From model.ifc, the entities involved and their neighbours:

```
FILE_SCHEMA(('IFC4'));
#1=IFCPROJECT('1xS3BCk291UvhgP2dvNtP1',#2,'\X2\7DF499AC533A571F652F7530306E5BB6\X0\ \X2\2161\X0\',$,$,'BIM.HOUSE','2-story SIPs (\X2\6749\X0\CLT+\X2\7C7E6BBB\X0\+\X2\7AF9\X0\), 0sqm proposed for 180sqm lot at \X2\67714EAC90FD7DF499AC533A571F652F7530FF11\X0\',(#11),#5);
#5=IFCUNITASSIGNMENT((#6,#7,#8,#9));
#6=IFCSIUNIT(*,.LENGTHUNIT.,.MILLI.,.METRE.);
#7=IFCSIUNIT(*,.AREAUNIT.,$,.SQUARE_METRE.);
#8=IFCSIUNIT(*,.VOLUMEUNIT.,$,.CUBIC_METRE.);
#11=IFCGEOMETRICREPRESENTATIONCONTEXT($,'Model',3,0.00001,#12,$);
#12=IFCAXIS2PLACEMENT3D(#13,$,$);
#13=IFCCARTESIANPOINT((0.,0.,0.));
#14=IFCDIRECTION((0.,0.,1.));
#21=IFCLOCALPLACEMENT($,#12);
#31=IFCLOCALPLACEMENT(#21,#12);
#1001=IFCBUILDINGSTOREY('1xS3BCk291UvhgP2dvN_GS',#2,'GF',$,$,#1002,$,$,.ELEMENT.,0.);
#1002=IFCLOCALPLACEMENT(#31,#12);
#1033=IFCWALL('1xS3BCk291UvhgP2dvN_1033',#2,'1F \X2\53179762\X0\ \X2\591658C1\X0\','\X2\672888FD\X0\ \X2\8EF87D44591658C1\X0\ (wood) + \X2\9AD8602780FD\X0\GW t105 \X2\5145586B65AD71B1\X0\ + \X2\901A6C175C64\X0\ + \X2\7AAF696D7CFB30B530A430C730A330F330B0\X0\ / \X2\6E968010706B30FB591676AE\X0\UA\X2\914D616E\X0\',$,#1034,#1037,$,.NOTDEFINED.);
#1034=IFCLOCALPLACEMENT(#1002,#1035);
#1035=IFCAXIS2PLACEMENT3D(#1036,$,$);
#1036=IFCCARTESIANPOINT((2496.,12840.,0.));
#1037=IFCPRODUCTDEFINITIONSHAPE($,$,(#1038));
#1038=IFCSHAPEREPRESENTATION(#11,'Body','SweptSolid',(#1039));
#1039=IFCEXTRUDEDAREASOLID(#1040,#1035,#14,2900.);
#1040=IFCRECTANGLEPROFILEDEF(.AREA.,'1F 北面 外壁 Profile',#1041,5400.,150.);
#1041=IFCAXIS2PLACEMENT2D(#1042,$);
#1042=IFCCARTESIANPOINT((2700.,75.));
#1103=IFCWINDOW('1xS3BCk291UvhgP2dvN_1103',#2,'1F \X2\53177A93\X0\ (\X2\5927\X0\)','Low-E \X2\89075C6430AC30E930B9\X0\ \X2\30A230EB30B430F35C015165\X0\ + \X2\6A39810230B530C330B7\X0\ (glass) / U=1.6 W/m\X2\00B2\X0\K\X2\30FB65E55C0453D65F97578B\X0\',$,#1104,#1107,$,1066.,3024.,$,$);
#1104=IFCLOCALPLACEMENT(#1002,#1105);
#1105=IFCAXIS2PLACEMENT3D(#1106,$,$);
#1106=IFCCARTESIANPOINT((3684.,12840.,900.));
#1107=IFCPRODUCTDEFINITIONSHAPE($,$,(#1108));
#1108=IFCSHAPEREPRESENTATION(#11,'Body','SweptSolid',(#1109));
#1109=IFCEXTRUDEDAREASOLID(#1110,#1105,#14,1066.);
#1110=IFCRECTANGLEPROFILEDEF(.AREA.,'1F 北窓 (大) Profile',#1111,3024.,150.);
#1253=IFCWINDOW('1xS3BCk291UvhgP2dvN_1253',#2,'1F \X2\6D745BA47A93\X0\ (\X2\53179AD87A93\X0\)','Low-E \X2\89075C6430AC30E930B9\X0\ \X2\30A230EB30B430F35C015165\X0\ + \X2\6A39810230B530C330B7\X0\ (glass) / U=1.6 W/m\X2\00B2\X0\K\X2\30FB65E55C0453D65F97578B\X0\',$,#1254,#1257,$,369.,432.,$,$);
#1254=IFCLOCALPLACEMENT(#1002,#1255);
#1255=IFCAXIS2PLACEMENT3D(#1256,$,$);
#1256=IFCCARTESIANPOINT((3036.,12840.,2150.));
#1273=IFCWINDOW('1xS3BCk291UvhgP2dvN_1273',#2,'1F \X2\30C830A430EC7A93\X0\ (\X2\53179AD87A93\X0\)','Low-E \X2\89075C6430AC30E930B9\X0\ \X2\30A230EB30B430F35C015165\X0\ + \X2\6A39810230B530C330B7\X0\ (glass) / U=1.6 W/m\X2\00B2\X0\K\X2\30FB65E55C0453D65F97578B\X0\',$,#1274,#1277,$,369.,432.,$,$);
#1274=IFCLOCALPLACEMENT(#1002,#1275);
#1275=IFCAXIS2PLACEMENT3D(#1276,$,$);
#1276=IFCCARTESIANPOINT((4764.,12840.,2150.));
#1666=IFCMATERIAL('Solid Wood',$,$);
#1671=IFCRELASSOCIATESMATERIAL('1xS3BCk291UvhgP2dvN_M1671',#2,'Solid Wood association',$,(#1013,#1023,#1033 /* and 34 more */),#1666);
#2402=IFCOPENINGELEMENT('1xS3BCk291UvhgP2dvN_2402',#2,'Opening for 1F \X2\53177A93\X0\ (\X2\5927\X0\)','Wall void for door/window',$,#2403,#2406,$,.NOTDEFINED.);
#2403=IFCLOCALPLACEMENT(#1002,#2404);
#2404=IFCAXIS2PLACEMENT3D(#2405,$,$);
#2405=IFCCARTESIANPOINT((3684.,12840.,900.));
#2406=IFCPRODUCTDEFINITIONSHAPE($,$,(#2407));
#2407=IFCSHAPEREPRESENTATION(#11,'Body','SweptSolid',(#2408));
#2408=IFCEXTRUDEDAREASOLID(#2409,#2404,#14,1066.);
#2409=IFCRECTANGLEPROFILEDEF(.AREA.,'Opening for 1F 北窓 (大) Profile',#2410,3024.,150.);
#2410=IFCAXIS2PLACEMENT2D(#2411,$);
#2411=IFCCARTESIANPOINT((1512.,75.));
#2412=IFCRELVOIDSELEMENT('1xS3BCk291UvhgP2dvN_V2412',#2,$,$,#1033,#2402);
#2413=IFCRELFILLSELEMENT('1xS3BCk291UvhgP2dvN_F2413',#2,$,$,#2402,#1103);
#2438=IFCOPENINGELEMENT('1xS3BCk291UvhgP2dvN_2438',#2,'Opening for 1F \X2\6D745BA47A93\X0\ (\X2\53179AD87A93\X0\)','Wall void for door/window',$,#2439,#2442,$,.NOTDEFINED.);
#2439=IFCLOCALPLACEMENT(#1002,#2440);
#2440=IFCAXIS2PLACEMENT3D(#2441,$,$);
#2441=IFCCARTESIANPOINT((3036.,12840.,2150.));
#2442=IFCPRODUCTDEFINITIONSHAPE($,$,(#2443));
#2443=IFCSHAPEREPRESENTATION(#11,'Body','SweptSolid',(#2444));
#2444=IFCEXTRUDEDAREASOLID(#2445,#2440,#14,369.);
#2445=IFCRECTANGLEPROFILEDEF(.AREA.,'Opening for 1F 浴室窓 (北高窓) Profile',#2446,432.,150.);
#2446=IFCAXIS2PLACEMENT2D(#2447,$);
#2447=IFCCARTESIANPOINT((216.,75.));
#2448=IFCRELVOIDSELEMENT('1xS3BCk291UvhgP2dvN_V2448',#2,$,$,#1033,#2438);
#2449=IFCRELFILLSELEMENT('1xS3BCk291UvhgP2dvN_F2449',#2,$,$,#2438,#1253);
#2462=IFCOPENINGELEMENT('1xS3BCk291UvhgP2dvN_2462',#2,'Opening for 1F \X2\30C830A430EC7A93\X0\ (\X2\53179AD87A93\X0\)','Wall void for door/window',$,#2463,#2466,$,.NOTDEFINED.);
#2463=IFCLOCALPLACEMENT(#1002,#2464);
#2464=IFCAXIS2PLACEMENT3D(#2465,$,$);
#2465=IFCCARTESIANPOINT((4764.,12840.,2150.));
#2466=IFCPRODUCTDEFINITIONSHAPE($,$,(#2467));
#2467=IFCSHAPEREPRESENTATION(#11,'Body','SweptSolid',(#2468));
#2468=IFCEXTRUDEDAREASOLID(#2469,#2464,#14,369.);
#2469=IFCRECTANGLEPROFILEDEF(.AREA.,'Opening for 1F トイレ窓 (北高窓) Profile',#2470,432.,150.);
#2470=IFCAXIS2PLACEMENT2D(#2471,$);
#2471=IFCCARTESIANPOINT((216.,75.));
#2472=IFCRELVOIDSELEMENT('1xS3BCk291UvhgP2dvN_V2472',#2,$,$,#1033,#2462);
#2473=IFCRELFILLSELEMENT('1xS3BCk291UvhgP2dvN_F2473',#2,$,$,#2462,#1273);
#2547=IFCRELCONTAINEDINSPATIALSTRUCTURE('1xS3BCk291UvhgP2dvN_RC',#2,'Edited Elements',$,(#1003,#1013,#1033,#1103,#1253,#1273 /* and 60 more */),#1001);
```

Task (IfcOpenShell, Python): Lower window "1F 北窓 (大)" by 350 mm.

```python
import numpy as np
import ifcopenshell
import ifcopenshell.api.geometry
import ifcopenshell.util.placement
import ifcopenshell.util.unit

model = ifcopenshell.open("model.ifc")
unit_scale = ifcopenshell.util.unit.calculate_unit_scale(model)

window = model.by_guid("1xS3BCk291UvhgP2dvN_1103")
opening = window.FillsVoids[0].RelatingOpeningElement
dz = -0.35 / unit_scale

shift = np.array([0.0, 0.0, dz])
# The window is not placed relative to its opening, so move both.
for product in (opening, window):
    matrix = ifcopenshell.util.placement.get_local_placement(product.ObjectPlacement)
    matrix[:3, 3] += shift
    ifcopenshell.api.geometry.edit_object_placement(model, product=product, matrix=matrix, is_si=False)

print(f"moved by {dz * unit_scale:+.3f} m")

model.write("model_edited.ifc")
```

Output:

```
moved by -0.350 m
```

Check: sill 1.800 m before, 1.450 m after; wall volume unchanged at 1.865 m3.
